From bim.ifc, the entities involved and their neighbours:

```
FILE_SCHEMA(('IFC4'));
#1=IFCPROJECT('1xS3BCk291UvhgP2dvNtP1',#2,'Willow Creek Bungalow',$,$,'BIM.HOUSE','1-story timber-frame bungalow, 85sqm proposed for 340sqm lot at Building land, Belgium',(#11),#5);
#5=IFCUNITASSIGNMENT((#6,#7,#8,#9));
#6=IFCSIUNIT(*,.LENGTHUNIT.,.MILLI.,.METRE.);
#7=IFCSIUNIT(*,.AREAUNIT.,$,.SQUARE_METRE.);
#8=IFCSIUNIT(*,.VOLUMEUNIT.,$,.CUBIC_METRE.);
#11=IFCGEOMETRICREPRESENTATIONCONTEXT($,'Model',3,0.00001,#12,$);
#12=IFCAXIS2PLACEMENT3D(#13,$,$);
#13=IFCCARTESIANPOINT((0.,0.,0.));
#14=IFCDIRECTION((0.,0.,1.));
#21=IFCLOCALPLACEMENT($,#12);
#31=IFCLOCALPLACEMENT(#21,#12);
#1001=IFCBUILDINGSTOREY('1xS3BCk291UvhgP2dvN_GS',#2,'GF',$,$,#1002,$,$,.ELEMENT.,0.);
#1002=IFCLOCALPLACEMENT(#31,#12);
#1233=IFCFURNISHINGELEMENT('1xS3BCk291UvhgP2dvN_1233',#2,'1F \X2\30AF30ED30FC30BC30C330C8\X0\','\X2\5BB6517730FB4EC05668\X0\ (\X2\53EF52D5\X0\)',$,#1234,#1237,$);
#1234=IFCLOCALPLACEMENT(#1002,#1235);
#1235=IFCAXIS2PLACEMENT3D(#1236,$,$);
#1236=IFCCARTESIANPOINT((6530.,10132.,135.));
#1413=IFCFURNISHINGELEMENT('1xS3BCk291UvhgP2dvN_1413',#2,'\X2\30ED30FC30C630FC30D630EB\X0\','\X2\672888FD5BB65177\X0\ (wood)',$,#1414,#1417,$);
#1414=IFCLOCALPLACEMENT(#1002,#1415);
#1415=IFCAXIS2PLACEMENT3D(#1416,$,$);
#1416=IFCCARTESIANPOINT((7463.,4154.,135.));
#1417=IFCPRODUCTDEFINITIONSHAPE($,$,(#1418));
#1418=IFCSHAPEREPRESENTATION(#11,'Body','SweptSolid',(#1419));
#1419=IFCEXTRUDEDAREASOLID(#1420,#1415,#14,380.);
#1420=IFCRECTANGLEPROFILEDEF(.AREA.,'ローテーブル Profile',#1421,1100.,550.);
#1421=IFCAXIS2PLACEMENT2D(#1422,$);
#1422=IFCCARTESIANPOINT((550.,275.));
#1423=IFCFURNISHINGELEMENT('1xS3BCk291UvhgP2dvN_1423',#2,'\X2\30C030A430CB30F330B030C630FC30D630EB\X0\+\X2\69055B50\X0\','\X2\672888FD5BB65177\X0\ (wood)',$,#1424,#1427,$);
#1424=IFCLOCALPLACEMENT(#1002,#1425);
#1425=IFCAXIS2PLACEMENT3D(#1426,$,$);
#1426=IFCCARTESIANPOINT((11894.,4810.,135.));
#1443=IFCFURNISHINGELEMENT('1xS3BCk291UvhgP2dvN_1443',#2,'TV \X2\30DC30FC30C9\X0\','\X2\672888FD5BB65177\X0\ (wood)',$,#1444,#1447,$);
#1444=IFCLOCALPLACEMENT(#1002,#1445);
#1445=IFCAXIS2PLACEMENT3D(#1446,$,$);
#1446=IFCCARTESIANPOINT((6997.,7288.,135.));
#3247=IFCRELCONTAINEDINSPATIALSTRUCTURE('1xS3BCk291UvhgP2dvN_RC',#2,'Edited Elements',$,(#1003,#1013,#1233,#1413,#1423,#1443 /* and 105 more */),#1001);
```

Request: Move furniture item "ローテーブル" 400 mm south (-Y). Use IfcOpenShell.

```python
import ifcopenshell
import ifcopenshell.api.geometry
import ifcopenshell.util.placement

model = ifcopenshell.open("bim.ifc")

item = model.by_guid("1xS3BCk291UvhgP2dvN_1413")
matrix = ifcopenshell.util.placement.get_local_placement(item.ObjectPlacement)
matrix[1, 3] -= 400.0
ifcopenshell.api.geometry.edit_object_placement(model, product=item, matrix=matrix, is_si=False)

print(ifcopenshell.util.placement.get_local_placement(item.ObjectPlacement).round(3) + 0.0)

model.write("bim-out.ifc")
```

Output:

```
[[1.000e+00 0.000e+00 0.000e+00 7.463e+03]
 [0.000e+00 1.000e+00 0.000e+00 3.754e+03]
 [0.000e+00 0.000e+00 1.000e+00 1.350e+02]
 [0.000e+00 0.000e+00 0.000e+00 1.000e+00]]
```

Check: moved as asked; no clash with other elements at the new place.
